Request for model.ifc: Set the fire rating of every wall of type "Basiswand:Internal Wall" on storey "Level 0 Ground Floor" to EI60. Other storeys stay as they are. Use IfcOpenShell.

First a look at what the model holds.

```python
import ifcopenshell
import ifcopenshell.util.element

model = ifcopenshell.open("model.ifc")
print(model.schema)
storey = next(s for s in model.by_type("IfcBuildingStorey") if s.Name == "Level 0 Ground Floor")
walls = [e for e in ifcopenshell.util.element.get_decomposition(storey) if e.is_a("IfcWall")]
seen = {}
for e in walls:
    element_type = ifcopenshell.util.element.get_type(e)
    key = (element_type.Name if element_type != e and element_type else None, ifcopenshell.util.element.get_pset(e, "Pset_WallCommon", "FireRating"))
    seen[key] = seen.get(key, 0) + 1
for (name, value), count in sorted(seen.items(), key=str):
    print(count, "x", name, "|", value)
```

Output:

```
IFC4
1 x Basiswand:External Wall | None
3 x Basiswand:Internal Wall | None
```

```python
import ifcopenshell
import ifcopenshell.api.pset
import ifcopenshell.util.element

model = ifcopenshell.open("model.ifc")

storey = next(s for s in model.by_type("IfcBuildingStorey") if s.Name == "Level 0 Ground Floor")
walls = [e for e in ifcopenshell.util.element.get_decomposition(storey) if e.is_a("IfcWall")]

count = 0
for e in walls:
    element_type = ifcopenshell.util.element.get_type(e)
    if element_type in (None, e) or element_type.Name != "Basiswand:Internal Wall":
        continue
    # add_pset returns the element's existing set when there is one.
    pset = ifcopenshell.api.pset.add_pset(model, product=e, name="Pset_WallCommon")
    ifcopenshell.api.pset.edit_pset(model, pset=pset, properties={"FireRating": "EI60"})
    count += 1

print(count, "walls updated")

model.write("model-out.ifc")
```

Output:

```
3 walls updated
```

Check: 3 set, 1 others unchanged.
